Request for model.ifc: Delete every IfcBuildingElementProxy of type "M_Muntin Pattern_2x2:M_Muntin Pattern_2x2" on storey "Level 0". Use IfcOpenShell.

First a look at what the model holds.

```python
import ifcopenshell
import ifcopenshell.util.element

model = ifcopenshell.open("model.ifc")
print(model.schema)
storey = next(s for s in model.by_type("IfcBuildingStorey") if s.Name == "Level 0")
proxies = [e for e in ifcopenshell.util.element.get_decomposition(storey) if e.is_a("IfcBuildingElementProxy")]
seen = {}
for e in proxies:
    element_type = ifcopenshell.util.element.get_type(e)
    name = element_type.Name if element_type not in (None, e) else None
    seen[name] = seen.get(name, 0) + 1
for name, count in sorted(seen.items(), key=str):
    print(count, "x", name)
```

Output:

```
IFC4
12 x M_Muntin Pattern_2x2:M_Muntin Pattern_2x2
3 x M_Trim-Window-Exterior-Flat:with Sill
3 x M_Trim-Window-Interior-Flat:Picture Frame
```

```python
import ifcopenshell
import ifcopenshell.api.root
import ifcopenshell.util.element

model = ifcopenshell.open("model.ifc")

storey = next(s for s in model.by_type("IfcBuildingStorey") if s.Name == "Level 0")
proxies = [e for e in ifcopenshell.util.element.get_decomposition(storey) if e.is_a("IfcBuildingElementProxy")]
targets = [e for e in proxies if (t := ifcopenshell.util.element.get_type(e)) not in (None, e) and t.Name == "M_Muntin Pattern_2x2:M_Muntin Pattern_2x2"]

for e in targets:
    ifcopenshell.api.root.remove_product(model, product=e)
print(len(targets), "removed")

model.write("model_updated.ifc")
```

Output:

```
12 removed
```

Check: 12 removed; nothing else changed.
